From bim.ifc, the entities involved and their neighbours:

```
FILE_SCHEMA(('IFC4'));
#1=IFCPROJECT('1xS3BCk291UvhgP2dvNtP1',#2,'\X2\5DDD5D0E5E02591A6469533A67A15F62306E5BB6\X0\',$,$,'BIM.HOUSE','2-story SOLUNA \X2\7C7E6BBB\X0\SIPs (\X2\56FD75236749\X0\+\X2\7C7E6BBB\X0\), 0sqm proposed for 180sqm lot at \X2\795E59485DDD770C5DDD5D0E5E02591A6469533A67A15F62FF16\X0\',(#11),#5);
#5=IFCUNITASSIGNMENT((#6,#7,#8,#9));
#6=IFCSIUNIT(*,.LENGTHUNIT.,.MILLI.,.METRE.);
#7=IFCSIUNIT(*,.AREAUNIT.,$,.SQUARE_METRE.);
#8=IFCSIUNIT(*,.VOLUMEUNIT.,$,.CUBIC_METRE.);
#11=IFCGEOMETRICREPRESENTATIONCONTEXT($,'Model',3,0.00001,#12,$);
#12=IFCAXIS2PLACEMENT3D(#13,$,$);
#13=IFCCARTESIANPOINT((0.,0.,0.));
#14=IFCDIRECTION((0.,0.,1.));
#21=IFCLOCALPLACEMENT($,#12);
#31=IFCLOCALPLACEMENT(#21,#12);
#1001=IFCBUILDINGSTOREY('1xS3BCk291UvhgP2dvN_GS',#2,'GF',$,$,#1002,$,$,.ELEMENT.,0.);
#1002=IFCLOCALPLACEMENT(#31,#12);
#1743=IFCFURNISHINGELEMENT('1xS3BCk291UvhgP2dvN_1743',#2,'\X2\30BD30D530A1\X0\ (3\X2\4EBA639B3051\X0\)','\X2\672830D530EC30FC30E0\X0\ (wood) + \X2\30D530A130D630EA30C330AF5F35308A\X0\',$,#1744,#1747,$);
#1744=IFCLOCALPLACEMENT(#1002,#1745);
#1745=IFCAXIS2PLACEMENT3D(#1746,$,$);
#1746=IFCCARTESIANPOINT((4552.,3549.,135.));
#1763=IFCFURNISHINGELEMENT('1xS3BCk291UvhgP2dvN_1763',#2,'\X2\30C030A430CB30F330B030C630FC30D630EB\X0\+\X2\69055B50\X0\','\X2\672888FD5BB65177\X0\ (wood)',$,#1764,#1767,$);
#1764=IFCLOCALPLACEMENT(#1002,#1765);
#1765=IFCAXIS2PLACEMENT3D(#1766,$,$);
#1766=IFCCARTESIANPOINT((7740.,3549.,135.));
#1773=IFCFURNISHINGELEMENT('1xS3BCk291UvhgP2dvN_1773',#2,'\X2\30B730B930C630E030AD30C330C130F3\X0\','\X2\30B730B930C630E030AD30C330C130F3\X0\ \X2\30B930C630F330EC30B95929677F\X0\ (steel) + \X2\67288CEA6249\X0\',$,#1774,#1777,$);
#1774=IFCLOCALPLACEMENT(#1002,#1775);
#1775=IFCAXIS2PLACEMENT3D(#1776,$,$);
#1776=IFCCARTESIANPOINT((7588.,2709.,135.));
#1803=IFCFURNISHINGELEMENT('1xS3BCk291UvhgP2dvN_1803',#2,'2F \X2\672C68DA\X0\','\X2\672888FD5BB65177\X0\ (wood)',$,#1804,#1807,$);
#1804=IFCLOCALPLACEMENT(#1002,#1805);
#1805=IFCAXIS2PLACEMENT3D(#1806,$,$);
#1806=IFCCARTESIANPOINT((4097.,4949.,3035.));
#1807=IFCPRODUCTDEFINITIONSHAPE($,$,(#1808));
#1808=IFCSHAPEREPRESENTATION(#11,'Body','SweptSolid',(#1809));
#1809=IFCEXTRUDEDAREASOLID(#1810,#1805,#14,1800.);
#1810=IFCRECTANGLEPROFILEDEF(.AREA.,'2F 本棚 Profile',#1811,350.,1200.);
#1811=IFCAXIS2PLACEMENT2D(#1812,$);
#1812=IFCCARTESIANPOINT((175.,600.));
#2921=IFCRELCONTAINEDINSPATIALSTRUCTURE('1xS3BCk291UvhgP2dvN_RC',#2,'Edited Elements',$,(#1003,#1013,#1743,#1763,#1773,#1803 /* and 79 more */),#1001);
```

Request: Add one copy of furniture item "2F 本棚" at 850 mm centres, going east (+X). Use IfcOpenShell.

```python
import numpy as np
import ifcopenshell
import ifcopenshell.api.geometry
import ifcopenshell.api.root
import ifcopenshell.util.element
import ifcopenshell.util.placement
import ifcopenshell.util.unit

model = ifcopenshell.open("bim.ifc")
unit_scale = ifcopenshell.util.unit.calculate_unit_scale(model)


def reuse_history(source, copy):
    """copy_class also copies each property set's owner history, people and application; keep the originals."""
    for rel in copy.IsDefinedBy:
        if rel.is_a("IfcRelDefinesByProperties") and (history := rel.RelatingPropertyDefinition.OwnerHistory):
            rel.RelatingPropertyDefinition.OwnerHistory = source.OwnerHistory
            ifcopenshell.util.element.remove_deep2(model, history)


source = model.by_guid("1xS3BCk291UvhgP2dvN_1803")
base = ifcopenshell.util.placement.get_local_placement(source.ObjectPlacement)
step = np.array([1.0, 0.0, 0.0]) * 0.85 / unit_scale

for i in range(1, 2):
    copy = ifcopenshell.api.root.copy_class(model, product=source)
    copy.Representation = ifcopenshell.util.element.copy_deep(
        model, source.Representation, exclude=["IfcGeometricRepresentationContext", "IfcRepresentationMap"]
    )
    reuse_history(source, copy)
    matrix = base.copy()
    matrix[:3, 3] += i * step
    print("added at", matrix[:3, 3].round(3) + 0.0)
    ifcopenshell.api.geometry.edit_object_placement(model, product=copy, matrix=matrix, is_si=False)

model.write("bim_v2.ifc")
```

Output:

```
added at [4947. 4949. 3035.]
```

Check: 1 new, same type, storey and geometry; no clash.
